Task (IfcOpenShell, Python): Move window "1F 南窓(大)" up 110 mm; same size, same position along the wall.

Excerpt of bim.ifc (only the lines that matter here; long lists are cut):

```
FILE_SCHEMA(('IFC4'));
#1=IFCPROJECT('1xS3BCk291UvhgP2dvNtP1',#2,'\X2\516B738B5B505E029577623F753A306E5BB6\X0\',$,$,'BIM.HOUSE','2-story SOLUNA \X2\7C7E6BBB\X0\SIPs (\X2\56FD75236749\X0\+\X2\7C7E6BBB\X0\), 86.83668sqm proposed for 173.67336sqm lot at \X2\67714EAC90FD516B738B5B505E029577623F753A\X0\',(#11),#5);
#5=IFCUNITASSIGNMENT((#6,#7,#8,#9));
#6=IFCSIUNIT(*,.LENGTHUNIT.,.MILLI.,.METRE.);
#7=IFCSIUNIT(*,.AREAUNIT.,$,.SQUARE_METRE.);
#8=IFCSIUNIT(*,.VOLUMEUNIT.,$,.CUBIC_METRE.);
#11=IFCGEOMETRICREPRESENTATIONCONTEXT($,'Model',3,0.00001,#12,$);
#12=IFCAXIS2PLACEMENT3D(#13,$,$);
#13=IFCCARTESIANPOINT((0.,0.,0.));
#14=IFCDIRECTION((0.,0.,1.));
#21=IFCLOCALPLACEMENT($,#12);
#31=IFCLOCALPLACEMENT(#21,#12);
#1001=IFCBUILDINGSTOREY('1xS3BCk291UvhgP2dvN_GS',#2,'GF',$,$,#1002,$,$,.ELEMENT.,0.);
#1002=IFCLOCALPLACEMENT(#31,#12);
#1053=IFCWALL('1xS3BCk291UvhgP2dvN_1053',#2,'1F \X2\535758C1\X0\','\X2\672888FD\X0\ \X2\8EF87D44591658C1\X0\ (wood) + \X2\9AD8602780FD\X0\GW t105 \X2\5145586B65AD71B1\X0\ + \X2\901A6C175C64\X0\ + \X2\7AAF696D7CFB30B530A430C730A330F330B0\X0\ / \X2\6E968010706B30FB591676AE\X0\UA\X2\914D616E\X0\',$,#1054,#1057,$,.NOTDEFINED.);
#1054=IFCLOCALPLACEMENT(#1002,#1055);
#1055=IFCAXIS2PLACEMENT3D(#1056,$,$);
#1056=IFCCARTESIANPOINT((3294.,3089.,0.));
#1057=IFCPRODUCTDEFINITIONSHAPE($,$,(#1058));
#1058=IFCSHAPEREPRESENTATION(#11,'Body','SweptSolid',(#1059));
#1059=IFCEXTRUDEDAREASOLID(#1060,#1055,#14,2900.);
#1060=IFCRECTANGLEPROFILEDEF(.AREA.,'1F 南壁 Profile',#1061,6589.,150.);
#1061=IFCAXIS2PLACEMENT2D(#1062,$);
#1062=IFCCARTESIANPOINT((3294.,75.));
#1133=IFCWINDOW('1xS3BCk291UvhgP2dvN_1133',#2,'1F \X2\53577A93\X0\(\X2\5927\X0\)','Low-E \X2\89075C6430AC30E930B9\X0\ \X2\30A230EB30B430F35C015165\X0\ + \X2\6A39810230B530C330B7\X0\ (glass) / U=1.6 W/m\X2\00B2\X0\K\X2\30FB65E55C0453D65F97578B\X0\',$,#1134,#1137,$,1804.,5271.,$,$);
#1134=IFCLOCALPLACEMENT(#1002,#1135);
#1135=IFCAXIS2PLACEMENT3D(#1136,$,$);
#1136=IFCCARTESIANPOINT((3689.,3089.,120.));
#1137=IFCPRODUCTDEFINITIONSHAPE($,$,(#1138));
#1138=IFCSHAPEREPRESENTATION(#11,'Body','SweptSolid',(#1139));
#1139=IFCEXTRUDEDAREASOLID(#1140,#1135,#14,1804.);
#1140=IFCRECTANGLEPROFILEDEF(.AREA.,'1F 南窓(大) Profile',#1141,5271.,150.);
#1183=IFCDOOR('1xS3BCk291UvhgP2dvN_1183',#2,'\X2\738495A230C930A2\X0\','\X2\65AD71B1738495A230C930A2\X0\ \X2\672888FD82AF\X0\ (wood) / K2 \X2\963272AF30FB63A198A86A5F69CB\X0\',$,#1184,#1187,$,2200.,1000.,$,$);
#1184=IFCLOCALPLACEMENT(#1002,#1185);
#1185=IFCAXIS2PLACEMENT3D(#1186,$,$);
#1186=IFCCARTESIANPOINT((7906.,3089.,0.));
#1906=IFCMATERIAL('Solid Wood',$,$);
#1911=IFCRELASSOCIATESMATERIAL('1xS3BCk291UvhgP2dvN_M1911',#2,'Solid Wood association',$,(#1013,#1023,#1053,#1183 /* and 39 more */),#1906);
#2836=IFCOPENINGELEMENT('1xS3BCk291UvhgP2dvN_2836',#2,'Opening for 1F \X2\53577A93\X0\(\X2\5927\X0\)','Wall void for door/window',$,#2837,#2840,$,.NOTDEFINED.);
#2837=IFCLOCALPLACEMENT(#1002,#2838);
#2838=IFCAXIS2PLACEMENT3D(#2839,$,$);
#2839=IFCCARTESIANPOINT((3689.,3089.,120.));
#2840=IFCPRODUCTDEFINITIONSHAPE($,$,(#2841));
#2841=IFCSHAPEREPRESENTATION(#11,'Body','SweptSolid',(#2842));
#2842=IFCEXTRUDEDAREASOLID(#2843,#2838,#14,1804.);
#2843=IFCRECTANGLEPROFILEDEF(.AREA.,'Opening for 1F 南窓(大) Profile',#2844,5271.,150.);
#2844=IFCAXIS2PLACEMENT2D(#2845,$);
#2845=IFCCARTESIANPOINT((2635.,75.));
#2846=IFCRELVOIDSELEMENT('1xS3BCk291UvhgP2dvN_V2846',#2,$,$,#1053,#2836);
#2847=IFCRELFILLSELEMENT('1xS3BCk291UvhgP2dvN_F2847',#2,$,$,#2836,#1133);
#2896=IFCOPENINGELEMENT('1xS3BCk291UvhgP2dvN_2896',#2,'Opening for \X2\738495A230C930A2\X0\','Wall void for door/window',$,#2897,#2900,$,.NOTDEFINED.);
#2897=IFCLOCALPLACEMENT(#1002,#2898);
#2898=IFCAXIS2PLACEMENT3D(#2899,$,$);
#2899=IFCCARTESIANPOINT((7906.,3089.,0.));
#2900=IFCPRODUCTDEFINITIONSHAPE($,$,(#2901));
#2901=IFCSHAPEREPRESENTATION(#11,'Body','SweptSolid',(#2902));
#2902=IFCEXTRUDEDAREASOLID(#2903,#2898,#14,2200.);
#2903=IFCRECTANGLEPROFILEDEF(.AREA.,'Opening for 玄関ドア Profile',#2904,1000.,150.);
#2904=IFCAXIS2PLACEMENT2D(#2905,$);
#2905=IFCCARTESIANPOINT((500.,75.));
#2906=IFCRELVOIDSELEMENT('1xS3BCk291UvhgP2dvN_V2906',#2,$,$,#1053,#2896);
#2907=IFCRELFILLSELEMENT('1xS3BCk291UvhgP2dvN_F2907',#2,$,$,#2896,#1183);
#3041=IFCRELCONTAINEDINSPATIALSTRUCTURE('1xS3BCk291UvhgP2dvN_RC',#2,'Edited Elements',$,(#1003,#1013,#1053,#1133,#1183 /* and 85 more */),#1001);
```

```python
import numpy as np
import ifcopenshell
import ifcopenshell.api.geometry
import ifcopenshell.util.placement
import ifcopenshell.util.unit

model = ifcopenshell.open("bim.ifc")
unit_scale = ifcopenshell.util.unit.calculate_unit_scale(model)

window = model.by_guid("1xS3BCk291UvhgP2dvN_1133")
opening = window.FillsVoids[0].RelatingOpeningElement
dz = 0.11 / unit_scale

shift = np.array([0.0, 0.0, dz])
# The window is not placed relative to its opening, so move both.
for product in (opening, window):
    matrix = ifcopenshell.util.placement.get_local_placement(product.ObjectPlacement)
    matrix[:3, 3] += shift
    ifcopenshell.api.geometry.edit_object_placement(model, product=product, matrix=matrix, is_si=False)

print(f"moved by {dz * unit_scale:+.3f} m")

model.write("bim-out.ifc")
```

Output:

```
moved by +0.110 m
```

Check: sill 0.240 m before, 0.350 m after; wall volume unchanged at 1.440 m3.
